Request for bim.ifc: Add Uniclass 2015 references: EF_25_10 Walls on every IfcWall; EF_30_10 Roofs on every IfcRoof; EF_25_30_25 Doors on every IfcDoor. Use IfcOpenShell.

First a look at what the model holds.

```python
import ifcopenshell

model = ifcopenshell.open("bim.ifc")
print(model.schema)
print("classifications:", [c.Name for c in model.by_type("IfcClassification")])
for ifc_class in ("IfcDoor", "IfcRoof", "IfcStair", "IfcWall", "IfcWindow"):
    print(ifc_class, len(model.by_type(ifc_class)))
```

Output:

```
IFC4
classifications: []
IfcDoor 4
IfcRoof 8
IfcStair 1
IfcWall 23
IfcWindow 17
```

```python
import ifcopenshell
import ifcopenshell.api.classification

model = ifcopenshell.open("bim.ifc")

system = ifcopenshell.api.classification.add_classification(model, classification="Uniclass 2015")

codes = {
    "IfcWall": ("EF_25_10", "Walls"),
    "IfcRoof": ("EF_30_10", "Roofs"),
    "IfcDoor": ("EF_25_30_25", "Doors"),
}
for ifc_class, (code, name) in codes.items():
    products = model.by_type(ifc_class)
    ifcopenshell.api.classification.add_reference(
        model, products=products, classification=system, identification=code, name=name
    )
    print(code, len(products))

model.write("bim-out.ifc")
```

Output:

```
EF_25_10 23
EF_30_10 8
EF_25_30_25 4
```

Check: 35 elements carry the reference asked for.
